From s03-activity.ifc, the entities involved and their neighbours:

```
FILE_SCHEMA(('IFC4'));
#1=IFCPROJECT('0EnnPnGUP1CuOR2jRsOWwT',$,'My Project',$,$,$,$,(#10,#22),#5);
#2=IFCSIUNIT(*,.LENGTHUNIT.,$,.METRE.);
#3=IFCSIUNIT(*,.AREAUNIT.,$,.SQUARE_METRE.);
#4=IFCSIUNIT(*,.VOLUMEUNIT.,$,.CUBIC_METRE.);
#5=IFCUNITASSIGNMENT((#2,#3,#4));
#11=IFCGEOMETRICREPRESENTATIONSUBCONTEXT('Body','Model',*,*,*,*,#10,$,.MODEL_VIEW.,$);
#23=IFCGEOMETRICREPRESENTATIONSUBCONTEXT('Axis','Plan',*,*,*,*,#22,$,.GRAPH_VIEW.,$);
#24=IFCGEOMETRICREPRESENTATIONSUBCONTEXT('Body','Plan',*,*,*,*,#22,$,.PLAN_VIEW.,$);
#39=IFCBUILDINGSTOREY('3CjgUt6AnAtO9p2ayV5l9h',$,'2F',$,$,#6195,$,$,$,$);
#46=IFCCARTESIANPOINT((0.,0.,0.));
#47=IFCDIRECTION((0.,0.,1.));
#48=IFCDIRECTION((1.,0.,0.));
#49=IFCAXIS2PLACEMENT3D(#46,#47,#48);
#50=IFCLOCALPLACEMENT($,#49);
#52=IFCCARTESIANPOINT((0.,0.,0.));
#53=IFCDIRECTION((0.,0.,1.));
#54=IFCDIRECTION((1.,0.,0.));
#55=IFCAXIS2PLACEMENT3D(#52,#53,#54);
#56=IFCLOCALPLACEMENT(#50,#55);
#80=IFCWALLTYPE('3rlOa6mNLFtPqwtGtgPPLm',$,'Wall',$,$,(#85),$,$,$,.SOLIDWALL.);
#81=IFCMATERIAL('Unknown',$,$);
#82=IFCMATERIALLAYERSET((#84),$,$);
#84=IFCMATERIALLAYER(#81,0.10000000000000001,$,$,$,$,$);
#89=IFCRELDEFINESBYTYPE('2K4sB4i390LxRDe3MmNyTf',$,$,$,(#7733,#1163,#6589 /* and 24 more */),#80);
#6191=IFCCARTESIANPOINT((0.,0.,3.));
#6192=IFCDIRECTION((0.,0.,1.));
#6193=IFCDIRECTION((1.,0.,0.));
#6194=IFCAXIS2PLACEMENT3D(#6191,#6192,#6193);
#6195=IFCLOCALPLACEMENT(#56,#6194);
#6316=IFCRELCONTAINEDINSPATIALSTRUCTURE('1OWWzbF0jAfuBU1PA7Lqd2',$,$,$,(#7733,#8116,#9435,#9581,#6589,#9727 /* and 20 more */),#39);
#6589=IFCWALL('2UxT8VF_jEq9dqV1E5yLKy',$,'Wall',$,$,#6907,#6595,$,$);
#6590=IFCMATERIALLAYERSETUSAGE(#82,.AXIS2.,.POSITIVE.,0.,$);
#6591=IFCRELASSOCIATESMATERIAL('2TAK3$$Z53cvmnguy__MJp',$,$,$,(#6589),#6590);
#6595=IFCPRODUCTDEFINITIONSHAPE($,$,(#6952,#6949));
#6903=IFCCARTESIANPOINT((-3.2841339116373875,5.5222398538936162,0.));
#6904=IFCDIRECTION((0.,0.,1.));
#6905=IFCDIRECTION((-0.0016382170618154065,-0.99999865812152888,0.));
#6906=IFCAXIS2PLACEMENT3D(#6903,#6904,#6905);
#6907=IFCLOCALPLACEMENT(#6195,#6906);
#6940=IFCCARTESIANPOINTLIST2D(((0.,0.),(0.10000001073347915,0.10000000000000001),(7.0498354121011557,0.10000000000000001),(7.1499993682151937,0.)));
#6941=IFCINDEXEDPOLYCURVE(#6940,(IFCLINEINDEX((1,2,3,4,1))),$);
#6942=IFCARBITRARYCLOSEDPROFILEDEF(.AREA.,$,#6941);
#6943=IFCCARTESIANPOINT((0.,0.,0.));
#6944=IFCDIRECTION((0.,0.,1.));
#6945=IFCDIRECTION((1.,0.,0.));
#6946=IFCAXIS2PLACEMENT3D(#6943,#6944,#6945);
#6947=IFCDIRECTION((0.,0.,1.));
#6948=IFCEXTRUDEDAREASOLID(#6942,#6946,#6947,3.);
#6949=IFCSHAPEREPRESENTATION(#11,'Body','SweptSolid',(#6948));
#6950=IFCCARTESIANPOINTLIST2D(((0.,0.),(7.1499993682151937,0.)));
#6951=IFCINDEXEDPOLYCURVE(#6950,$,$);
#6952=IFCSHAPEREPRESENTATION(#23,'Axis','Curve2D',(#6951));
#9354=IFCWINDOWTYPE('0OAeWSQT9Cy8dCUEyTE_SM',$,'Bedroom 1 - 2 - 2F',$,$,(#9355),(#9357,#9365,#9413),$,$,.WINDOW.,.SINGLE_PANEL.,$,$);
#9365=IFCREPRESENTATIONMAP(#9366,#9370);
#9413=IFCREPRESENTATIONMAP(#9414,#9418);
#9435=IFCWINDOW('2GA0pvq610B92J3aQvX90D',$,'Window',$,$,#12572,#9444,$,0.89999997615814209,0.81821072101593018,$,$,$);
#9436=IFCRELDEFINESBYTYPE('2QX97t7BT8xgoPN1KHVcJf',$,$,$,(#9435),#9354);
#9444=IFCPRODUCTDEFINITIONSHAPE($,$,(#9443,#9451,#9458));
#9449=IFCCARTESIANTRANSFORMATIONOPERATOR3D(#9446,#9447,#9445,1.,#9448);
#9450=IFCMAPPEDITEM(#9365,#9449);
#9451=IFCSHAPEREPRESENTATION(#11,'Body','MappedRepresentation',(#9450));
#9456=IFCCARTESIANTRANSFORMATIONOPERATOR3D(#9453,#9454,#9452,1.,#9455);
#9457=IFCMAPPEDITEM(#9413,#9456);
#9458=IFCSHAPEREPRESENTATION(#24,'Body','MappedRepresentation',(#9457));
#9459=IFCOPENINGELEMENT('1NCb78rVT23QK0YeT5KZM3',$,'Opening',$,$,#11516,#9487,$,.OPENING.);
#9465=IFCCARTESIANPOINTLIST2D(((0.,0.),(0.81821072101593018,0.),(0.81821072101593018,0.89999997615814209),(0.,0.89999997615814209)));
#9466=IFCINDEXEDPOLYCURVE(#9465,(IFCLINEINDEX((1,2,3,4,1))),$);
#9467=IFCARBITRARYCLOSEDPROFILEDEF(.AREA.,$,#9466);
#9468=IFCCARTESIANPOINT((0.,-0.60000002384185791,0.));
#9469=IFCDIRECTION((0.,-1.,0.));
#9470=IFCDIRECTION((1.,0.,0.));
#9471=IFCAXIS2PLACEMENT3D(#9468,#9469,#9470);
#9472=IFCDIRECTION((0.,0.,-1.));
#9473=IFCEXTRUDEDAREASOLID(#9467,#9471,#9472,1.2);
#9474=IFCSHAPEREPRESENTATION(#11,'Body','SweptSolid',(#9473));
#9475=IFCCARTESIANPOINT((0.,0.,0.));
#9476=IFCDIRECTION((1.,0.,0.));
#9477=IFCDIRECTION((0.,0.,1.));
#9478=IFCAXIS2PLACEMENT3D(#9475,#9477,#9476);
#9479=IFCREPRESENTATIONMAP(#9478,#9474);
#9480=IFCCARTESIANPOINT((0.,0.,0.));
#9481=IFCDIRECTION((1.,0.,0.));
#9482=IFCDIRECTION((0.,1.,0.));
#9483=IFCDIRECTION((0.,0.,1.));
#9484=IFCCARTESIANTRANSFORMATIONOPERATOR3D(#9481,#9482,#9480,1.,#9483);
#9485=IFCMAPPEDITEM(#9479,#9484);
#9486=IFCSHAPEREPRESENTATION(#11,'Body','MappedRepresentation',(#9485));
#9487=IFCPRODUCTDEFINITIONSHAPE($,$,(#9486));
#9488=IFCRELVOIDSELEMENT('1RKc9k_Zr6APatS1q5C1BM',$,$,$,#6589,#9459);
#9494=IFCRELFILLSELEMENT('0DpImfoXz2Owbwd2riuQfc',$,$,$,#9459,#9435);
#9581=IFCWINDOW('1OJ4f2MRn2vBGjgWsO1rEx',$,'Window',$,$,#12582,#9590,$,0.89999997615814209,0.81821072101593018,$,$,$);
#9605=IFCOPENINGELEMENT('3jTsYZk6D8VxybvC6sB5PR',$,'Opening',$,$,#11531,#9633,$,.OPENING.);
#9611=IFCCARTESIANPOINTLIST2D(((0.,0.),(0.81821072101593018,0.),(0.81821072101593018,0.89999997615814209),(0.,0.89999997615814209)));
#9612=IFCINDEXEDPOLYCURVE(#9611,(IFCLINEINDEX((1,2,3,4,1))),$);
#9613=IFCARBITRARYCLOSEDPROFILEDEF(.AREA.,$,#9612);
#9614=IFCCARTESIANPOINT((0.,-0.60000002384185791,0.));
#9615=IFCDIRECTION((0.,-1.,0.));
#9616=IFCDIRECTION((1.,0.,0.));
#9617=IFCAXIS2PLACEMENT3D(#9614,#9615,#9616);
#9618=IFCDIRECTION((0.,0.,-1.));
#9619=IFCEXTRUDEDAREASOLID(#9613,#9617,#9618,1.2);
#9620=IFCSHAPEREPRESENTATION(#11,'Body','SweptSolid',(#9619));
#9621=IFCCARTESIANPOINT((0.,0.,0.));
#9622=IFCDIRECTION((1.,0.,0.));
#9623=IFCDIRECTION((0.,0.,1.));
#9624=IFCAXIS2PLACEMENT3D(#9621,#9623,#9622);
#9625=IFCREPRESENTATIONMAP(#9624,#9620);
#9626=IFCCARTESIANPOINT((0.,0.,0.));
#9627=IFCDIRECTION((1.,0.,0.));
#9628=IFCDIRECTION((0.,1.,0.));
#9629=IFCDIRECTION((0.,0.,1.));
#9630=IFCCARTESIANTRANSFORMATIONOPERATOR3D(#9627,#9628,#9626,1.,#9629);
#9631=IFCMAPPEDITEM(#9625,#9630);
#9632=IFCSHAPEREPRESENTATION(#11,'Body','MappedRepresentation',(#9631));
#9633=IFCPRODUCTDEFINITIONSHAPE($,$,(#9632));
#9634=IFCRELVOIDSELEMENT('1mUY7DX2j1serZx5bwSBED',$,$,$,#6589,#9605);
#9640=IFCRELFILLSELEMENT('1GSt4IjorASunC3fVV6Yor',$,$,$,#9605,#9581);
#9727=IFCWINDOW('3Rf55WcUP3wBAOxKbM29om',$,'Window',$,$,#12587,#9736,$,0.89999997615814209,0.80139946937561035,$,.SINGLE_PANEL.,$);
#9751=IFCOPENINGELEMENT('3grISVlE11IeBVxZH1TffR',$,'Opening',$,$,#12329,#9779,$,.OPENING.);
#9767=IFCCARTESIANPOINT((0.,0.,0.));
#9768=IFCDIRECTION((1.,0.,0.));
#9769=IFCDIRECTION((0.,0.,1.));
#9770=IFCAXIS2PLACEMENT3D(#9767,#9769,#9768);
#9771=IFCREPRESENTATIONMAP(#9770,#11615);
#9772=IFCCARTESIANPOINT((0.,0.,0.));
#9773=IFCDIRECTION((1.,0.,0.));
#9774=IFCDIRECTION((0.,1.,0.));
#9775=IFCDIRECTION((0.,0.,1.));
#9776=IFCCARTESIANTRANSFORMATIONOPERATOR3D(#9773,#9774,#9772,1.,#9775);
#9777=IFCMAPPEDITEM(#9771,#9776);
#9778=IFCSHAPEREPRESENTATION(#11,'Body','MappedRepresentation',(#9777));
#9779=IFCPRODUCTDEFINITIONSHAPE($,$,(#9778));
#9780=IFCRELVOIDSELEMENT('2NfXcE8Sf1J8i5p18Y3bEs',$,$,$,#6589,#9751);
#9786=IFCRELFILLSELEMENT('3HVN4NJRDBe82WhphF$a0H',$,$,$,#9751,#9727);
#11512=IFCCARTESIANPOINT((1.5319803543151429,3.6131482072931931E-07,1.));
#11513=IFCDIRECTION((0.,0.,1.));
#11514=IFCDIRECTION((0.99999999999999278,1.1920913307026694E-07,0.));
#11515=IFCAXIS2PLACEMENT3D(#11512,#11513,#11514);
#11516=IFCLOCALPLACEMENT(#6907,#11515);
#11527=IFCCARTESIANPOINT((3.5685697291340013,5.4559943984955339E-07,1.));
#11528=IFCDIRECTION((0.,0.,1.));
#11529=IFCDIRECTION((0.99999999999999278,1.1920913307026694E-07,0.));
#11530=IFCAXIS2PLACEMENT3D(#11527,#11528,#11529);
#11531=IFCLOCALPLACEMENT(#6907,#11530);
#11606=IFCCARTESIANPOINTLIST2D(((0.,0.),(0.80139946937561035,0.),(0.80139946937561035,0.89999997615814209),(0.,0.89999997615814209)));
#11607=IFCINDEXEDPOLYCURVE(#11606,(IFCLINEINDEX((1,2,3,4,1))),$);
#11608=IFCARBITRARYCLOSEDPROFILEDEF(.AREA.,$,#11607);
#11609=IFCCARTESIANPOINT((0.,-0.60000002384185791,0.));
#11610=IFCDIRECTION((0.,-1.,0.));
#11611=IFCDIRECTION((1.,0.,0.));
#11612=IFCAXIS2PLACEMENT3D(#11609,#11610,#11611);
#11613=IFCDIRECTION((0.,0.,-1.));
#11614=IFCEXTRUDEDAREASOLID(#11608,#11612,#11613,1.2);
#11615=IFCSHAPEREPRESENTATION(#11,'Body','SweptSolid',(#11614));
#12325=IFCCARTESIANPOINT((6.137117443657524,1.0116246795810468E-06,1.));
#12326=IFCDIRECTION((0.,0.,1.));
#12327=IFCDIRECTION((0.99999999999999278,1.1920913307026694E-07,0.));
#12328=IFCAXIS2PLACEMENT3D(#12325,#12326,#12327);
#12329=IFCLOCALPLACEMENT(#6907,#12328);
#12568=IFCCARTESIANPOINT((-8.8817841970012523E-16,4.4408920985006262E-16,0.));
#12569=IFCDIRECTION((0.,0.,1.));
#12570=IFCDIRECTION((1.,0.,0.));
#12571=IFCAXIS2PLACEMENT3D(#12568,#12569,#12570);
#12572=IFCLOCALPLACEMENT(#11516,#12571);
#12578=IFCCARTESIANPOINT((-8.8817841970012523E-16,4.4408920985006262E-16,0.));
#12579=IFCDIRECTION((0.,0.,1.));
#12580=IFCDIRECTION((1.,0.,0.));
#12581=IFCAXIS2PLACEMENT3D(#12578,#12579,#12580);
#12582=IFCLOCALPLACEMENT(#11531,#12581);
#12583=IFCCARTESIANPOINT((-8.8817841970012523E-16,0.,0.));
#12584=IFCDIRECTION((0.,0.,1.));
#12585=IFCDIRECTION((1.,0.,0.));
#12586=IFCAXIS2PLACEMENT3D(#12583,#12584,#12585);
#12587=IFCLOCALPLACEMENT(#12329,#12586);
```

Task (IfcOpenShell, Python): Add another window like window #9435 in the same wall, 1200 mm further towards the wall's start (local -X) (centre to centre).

```python
import ifcopenshell
import ifcopenshell.api.feature
import ifcopenshell.api.geometry
import ifcopenshell.api.root
import ifcopenshell.geom
import ifcopenshell.util.element
import ifcopenshell.util.placement
import ifcopenshell.util.shape
import ifcopenshell.util.unit

model = ifcopenshell.open("s03-activity.ifc")
unit_scale = ifcopenshell.util.unit.calculate_unit_scale(model)
settings = ifcopenshell.geom.settings()


def volume(element):
    """Net volume in cubic metres, openings subtracted."""
    shape = ifcopenshell.geom.create_shape(settings, element)
    return ifcopenshell.util.shape.get_volume(shape.geometry)


window = model.by_id(9435)
opening = window.FillsVoids[0].RelatingOpeningElement
wall = opening.VoidsElements[0].RelatingBuildingElement
before = volume(wall)
shift = ifcopenshell.util.placement.get_local_placement(wall.ObjectPlacement)[:3, 0] * -1.2 / unit_scale

# copy_class copies the void relationship, type, container and properties, but no geometry.
new_opening = ifcopenshell.api.root.copy_class(model, product=opening)
new_opening.Representation = ifcopenshell.util.element.copy_deep(
    model, opening.Representation, exclude=["IfcGeometricRepresentationContext", "IfcRepresentationMap"]
)
new_window = ifcopenshell.api.root.copy_class(model, product=window)
new_window.Representation = ifcopenshell.util.element.copy_deep(
    model, window.Representation, exclude=["IfcGeometricRepresentationContext", "IfcRepresentationMap"]
)
ifcopenshell.api.feature.add_filling(model, opening=new_opening, element=new_window)

for old, new in ((opening, new_opening), (window, new_window)):
    matrix = ifcopenshell.util.placement.get_local_placement(old.ObjectPlacement)
    matrix[:3, 3] += shift
    ifcopenshell.api.geometry.edit_object_placement(model, product=new, matrix=matrix, is_si=False)

after = volume(wall)

print(f"wall volume {before:.3f} -> {after:.3f} m3")

model.write("s03-activity_updated.ifc")
```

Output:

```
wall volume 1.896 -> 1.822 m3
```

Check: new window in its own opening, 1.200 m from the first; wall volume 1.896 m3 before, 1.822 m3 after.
